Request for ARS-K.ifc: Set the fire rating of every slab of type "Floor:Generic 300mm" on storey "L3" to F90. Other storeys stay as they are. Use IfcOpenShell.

First a look at what the model holds.

```python
import ifcopenshell
import ifcopenshell.util.element

model = ifcopenshell.open("ARS-K.ifc")
print(model.schema)
storey = next(s for s in model.by_type("IfcBuildingStorey") if s.Name == "L3")
slabs = [e for e in ifcopenshell.util.element.get_decomposition(storey) if e.is_a("IfcSlab")]
seen = {}
for e in slabs:
    element_type = ifcopenshell.util.element.get_type(e)
    key = (element_type.Name if element_type != e and element_type else None, ifcopenshell.util.element.get_pset(e, "Pset_SlabCommon", "FireRating"))
    seen[key] = seen.get(key, 0) + 1
for (name, value), count in sorted(seen.items(), key=str):
    print(count, "x", name, "|", value)
```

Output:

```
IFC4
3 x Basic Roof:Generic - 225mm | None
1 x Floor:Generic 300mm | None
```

```python
import ifcopenshell
import ifcopenshell.api.pset
import ifcopenshell.util.element

model = ifcopenshell.open("ARS-K.ifc")

storey = next(s for s in model.by_type("IfcBuildingStorey") if s.Name == "L3")
slabs = [e for e in ifcopenshell.util.element.get_decomposition(storey) if e.is_a("IfcSlab")]

count = 0
for e in slabs:
    element_type = ifcopenshell.util.element.get_type(e)
    if element_type in (None, e) or element_type.Name != "Floor:Generic 300mm":
        continue
    # add_pset returns the element's existing set when there is one.
    pset = ifcopenshell.api.pset.add_pset(model, product=e, name="Pset_SlabCommon")
    ifcopenshell.api.pset.edit_pset(model, pset=pset, properties={"FireRating": "F90"})
    count += 1

print(count, "slabs updated")

model.write("ARS-K_v2.ifc")
```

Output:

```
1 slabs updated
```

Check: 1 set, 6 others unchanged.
